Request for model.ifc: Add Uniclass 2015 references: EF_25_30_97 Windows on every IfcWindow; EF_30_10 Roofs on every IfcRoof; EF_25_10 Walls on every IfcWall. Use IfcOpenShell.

First a look at what the model holds.

```python
import ifcopenshell

model = ifcopenshell.open("model.ifc")
print(model.schema)
print("classifications:", [c.Name for c in model.by_type("IfcClassification")])
for ifc_class in ("IfcDoor", "IfcRoof", "IfcStair", "IfcWall", "IfcWindow"):
    print(ifc_class, len(model.by_type(ifc_class)))
```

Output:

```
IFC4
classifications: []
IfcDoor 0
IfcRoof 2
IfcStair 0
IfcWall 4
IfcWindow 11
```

```python
import ifcopenshell
import ifcopenshell.api.classification

model = ifcopenshell.open("model.ifc")

system = ifcopenshell.api.classification.add_classification(model, classification="Uniclass 2015")

codes = {
    "IfcWindow": ("EF_25_30_97", "Windows"),
    "IfcRoof": ("EF_30_10", "Roofs"),
    "IfcWall": ("EF_25_10", "Walls"),
}
for ifc_class, (code, name) in codes.items():
    products = model.by_type(ifc_class)
    ifcopenshell.api.classification.add_reference(
        model, products=products, classification=system, identification=code, name=name
    )
    print(code, len(products))

model.write("model_edited.ifc")
```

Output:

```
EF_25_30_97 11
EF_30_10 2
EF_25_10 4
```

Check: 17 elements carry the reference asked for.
